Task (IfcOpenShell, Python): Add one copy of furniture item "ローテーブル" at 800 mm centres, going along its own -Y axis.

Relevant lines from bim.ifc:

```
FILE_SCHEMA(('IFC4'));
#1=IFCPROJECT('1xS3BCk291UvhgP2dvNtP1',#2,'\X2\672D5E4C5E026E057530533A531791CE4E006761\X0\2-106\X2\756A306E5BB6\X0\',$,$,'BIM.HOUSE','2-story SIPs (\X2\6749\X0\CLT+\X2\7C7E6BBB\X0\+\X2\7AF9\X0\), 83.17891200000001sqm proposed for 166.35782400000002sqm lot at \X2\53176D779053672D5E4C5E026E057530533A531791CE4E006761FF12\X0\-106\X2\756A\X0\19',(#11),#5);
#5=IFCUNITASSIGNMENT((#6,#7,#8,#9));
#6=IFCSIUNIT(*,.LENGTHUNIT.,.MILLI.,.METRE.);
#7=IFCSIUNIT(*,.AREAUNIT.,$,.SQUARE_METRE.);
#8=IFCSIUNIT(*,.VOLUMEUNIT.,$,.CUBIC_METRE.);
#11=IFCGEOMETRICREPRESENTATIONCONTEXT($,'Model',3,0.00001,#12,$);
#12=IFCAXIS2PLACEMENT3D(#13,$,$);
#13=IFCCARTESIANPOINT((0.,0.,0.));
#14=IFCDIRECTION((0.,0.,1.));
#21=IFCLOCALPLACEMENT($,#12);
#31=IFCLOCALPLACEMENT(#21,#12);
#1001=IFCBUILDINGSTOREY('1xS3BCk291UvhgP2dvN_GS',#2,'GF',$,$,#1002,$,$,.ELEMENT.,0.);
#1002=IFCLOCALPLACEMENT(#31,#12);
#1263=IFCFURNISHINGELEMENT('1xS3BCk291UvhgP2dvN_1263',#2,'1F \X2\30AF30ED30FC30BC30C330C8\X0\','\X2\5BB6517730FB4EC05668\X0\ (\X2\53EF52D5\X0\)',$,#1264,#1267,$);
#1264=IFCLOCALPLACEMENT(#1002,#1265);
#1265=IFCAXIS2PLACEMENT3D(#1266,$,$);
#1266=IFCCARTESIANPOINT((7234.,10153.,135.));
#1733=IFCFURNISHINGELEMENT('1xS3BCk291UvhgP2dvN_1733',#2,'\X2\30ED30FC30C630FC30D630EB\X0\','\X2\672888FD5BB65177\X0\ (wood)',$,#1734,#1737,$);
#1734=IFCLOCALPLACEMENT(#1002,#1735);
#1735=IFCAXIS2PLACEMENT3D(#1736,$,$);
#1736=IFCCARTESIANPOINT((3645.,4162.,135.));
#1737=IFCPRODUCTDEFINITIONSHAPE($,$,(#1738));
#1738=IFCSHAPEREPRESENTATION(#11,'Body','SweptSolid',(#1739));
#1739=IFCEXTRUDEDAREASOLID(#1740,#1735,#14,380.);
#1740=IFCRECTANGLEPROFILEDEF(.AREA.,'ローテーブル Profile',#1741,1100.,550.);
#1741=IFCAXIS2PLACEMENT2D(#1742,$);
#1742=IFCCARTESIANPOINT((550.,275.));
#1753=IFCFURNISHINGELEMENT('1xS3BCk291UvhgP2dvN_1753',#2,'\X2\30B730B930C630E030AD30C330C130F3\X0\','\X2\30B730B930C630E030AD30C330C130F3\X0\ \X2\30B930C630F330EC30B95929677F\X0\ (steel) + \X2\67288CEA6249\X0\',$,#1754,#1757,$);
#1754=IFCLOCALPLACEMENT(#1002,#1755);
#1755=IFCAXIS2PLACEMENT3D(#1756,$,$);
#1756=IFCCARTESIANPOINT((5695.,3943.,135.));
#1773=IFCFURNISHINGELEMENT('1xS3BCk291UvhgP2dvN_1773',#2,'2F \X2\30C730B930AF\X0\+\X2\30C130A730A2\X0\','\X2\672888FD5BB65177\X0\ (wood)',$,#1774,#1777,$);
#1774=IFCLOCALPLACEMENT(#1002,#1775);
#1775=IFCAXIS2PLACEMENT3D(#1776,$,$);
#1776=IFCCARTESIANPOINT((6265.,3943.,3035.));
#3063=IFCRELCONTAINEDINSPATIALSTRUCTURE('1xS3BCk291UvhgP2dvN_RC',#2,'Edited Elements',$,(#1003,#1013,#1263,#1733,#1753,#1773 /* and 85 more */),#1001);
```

```python
import ifcopenshell
import ifcopenshell.api.geometry
import ifcopenshell.api.root
import ifcopenshell.util.element
import ifcopenshell.util.placement
import ifcopenshell.util.unit

model = ifcopenshell.open("bim.ifc")
unit_scale = ifcopenshell.util.unit.calculate_unit_scale(model)


def reuse_history(source, copy):
    """copy_class also copies each property set's owner history, people and application; keep the originals."""
    for rel in copy.IsDefinedBy:
        if rel.is_a("IfcRelDefinesByProperties") and (history := rel.RelatingPropertyDefinition.OwnerHistory):
            rel.RelatingPropertyDefinition.OwnerHistory = source.OwnerHistory
            ifcopenshell.util.element.remove_deep2(model, history)


source = model.by_guid("1xS3BCk291UvhgP2dvN_1733")
base = ifcopenshell.util.placement.get_local_placement(source.ObjectPlacement)
step = -base[:3, 1] * 0.8 / unit_scale

for i in range(1, 2):
    copy = ifcopenshell.api.root.copy_class(model, product=source)
    copy.Representation = ifcopenshell.util.element.copy_deep(
        model, source.Representation, exclude=["IfcGeometricRepresentationContext", "IfcRepresentationMap"]
    )
    reuse_history(source, copy)
    matrix = base.copy()
    matrix[:3, 3] += i * step
    print("added at", matrix[:3, 3].round(3) + 0.0)
    ifcopenshell.api.geometry.edit_object_placement(model, product=copy, matrix=matrix, is_si=False)

model.write("bim-out.ifc")
```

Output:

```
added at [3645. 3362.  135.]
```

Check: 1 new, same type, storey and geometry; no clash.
